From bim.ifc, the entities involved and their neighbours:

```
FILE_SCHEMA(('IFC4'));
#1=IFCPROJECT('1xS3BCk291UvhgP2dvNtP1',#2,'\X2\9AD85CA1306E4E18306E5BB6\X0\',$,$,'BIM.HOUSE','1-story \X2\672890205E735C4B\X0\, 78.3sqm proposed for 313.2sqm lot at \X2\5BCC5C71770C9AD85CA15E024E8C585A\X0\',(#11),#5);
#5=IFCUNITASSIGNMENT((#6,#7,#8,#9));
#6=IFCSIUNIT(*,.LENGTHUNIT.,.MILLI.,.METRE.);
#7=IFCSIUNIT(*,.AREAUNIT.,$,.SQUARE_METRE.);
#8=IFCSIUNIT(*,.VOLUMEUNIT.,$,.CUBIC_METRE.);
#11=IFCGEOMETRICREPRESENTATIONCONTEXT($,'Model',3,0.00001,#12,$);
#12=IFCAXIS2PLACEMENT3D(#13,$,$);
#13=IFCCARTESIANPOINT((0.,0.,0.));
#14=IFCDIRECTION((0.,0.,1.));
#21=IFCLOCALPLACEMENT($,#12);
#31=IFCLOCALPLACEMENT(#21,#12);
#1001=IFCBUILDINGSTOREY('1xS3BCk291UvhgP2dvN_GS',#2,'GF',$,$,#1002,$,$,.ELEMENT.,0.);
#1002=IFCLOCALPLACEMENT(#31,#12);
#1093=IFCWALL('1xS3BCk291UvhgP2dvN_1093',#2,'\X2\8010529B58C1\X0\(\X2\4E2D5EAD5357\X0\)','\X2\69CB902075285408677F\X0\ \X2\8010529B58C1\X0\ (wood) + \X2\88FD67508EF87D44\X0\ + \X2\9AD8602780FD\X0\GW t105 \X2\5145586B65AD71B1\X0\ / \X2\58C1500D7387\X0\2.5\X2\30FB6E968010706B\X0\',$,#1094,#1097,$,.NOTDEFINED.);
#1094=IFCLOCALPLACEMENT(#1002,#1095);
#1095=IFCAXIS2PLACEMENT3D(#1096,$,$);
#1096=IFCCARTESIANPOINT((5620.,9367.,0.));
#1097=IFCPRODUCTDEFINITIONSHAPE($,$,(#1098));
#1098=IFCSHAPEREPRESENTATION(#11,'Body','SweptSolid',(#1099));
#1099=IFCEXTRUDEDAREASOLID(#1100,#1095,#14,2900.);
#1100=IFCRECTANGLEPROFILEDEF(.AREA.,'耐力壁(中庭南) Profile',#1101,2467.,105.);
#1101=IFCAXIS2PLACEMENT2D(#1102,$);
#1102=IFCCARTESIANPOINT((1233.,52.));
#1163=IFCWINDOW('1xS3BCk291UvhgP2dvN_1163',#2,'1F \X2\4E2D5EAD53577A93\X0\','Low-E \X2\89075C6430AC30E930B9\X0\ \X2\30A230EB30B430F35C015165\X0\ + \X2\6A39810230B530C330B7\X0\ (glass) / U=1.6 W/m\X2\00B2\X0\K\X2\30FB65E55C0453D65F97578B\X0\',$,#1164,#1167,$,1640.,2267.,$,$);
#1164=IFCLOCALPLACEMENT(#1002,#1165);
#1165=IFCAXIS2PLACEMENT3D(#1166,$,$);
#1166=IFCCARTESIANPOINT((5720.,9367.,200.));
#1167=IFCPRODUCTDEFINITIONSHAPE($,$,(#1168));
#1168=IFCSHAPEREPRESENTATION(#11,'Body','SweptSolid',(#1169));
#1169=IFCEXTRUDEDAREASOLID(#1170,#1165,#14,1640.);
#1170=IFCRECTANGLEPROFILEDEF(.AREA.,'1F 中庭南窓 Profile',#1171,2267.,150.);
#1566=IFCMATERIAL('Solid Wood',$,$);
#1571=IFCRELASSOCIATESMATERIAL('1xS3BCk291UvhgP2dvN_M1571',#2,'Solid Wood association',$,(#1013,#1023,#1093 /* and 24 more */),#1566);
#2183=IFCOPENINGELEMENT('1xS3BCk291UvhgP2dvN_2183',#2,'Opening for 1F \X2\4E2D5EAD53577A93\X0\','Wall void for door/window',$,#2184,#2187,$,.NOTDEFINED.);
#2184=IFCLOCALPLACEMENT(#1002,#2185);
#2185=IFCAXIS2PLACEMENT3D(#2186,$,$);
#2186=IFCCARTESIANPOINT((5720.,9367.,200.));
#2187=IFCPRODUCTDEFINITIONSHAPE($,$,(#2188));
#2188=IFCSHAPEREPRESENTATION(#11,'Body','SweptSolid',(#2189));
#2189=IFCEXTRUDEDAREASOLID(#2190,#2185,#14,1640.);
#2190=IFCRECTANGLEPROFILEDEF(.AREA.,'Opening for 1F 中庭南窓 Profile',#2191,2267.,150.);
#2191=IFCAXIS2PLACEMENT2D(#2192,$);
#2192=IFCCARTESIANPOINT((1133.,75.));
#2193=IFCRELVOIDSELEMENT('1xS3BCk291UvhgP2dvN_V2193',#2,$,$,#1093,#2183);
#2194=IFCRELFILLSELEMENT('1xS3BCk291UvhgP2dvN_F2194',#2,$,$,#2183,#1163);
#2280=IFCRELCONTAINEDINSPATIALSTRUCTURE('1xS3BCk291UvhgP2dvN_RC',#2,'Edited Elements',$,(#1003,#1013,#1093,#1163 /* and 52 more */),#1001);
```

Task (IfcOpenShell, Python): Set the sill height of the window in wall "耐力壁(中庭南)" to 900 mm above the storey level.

```python
import numpy as np
import ifcopenshell
import ifcopenshell.api.geometry
import ifcopenshell.geom
import ifcopenshell.util.element
import ifcopenshell.util.placement
import ifcopenshell.util.shape
import ifcopenshell.util.unit

model = ifcopenshell.open("bim.ifc")
unit_scale = ifcopenshell.util.unit.calculate_unit_scale(model)

window = model.by_guid("1xS3BCk291UvhgP2dvN_1163")
opening = window.FillsVoids[0].RelatingOpeningElement
storey = ifcopenshell.util.element.get_container(window, ifc_class="IfcBuildingStorey")
level = ifcopenshell.util.placement.get_local_placement(storey.ObjectPlacement)[2, 3]

# The opening's origin need not be at the sill, so measure its lowest point.
shape = ifcopenshell.geom.create_shape(ifcopenshell.geom.settings(), opening)
bottom = ifcopenshell.util.shape.get_shape_bottom_elevation(shape, shape.geometry) / unit_scale
dz = level + 0.9 / unit_scale - bottom

shift = np.array([0.0, 0.0, dz])
# The window is not placed relative to its opening, so move both.
for product in (opening, window):
    matrix = ifcopenshell.util.placement.get_local_placement(product.ObjectPlacement)
    matrix[:3, 3] += shift
    ifcopenshell.api.geometry.edit_object_placement(model, product=product, matrix=matrix, is_si=False)

print(f"moved by {dz * unit_scale:+.3f} m")

model.write("bim-out.ifc")
```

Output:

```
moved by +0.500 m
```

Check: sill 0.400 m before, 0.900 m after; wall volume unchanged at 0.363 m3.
